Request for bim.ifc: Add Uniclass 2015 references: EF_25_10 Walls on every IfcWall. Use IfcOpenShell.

First a look at what the model holds.

```python
import ifcopenshell

model = ifcopenshell.open("bim.ifc")
print(model.schema)
print("classifications:", [c.Name for c in model.by_type("IfcClassification")])
for ifc_class in ("IfcDoor", "IfcRoof", "IfcStair", "IfcWall", "IfcWindow"):
    print(ifc_class, len(model.by_type(ifc_class)))
```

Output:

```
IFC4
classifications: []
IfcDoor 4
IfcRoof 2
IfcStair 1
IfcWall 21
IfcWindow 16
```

```python
import ifcopenshell
import ifcopenshell.api.classification

model = ifcopenshell.open("bim.ifc")

system = ifcopenshell.api.classification.add_classification(model, classification="Uniclass 2015")

codes = {
    "IfcWall": ("EF_25_10", "Walls"),
}
for ifc_class, (code, name) in codes.items():
    products = model.by_type(ifc_class)
    ifcopenshell.api.classification.add_reference(
        model, products=products, classification=system, identification=code, name=name
    )
    print(code, len(products))

model.write("bim_updated.ifc")
```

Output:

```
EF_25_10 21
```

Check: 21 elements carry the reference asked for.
